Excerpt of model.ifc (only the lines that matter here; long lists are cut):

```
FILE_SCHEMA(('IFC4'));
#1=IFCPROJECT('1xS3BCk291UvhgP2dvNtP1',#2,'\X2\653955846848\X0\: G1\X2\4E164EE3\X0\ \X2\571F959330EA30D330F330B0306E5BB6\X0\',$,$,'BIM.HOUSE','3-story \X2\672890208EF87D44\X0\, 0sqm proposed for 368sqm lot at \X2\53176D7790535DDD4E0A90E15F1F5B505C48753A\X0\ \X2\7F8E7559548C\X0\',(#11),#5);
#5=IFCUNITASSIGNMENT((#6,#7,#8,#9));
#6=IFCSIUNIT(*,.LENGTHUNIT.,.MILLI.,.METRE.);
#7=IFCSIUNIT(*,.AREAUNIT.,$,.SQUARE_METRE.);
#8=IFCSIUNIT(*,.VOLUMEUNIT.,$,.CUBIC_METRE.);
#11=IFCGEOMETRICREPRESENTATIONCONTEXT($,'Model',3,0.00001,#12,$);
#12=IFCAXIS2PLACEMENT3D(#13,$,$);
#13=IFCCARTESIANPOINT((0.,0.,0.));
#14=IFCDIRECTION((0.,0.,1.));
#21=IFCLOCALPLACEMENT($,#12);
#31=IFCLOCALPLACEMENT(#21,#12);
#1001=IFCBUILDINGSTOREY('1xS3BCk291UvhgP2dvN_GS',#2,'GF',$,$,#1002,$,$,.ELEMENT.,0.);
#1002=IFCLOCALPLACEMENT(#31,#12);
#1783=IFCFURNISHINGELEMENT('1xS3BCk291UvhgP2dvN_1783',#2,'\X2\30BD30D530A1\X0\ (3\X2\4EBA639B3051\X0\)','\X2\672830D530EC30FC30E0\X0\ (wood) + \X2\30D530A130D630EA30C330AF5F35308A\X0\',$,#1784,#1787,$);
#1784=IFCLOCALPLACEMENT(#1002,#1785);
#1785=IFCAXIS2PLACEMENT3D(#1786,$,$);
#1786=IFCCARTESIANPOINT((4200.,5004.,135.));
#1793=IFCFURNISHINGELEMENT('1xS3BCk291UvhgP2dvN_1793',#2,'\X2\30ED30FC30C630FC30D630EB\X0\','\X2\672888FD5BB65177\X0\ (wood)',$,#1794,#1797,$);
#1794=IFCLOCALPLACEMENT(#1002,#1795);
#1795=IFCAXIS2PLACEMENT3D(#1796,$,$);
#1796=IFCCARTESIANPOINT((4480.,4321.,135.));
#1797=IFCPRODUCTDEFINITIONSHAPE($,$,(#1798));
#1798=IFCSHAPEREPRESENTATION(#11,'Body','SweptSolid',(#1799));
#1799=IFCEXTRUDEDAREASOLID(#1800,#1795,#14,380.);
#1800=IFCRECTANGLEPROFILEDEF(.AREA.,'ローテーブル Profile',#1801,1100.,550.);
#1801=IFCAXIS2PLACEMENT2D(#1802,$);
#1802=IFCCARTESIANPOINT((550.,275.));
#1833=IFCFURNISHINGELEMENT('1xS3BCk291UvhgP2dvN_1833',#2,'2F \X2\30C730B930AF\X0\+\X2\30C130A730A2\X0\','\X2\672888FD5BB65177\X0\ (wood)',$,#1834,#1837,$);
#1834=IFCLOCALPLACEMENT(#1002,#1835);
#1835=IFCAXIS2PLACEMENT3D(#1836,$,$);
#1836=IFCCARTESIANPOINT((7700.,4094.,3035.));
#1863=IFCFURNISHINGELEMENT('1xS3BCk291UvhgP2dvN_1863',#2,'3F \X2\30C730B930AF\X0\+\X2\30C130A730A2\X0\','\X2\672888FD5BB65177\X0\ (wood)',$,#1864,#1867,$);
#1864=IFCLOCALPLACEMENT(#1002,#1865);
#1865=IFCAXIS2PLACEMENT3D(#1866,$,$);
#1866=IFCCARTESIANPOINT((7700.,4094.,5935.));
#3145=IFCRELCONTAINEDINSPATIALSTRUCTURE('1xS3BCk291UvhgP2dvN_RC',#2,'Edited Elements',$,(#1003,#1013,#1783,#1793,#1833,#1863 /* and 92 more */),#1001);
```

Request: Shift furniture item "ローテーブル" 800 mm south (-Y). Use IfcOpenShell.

```python
import ifcopenshell
import ifcopenshell.api.geometry
import ifcopenshell.util.placement
import ifcopenshell.util.unit

model = ifcopenshell.open("model.ifc")
unit_scale = ifcopenshell.util.unit.calculate_unit_scale(model)

item = model.by_id(1793)
matrix = ifcopenshell.util.placement.get_local_placement(item.ObjectPlacement)
matrix[1, 3] -= 0.8 / unit_scale
ifcopenshell.api.geometry.edit_object_placement(model, product=item, matrix=matrix, is_si=False)

print(ifcopenshell.util.placement.get_local_placement(item.ObjectPlacement).round(3) + 0.0)

model.write("model_updated.ifc")
```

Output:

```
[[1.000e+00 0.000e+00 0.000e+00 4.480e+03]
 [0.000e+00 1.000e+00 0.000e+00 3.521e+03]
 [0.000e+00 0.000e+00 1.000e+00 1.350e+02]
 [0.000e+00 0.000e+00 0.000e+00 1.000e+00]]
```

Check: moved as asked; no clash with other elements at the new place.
